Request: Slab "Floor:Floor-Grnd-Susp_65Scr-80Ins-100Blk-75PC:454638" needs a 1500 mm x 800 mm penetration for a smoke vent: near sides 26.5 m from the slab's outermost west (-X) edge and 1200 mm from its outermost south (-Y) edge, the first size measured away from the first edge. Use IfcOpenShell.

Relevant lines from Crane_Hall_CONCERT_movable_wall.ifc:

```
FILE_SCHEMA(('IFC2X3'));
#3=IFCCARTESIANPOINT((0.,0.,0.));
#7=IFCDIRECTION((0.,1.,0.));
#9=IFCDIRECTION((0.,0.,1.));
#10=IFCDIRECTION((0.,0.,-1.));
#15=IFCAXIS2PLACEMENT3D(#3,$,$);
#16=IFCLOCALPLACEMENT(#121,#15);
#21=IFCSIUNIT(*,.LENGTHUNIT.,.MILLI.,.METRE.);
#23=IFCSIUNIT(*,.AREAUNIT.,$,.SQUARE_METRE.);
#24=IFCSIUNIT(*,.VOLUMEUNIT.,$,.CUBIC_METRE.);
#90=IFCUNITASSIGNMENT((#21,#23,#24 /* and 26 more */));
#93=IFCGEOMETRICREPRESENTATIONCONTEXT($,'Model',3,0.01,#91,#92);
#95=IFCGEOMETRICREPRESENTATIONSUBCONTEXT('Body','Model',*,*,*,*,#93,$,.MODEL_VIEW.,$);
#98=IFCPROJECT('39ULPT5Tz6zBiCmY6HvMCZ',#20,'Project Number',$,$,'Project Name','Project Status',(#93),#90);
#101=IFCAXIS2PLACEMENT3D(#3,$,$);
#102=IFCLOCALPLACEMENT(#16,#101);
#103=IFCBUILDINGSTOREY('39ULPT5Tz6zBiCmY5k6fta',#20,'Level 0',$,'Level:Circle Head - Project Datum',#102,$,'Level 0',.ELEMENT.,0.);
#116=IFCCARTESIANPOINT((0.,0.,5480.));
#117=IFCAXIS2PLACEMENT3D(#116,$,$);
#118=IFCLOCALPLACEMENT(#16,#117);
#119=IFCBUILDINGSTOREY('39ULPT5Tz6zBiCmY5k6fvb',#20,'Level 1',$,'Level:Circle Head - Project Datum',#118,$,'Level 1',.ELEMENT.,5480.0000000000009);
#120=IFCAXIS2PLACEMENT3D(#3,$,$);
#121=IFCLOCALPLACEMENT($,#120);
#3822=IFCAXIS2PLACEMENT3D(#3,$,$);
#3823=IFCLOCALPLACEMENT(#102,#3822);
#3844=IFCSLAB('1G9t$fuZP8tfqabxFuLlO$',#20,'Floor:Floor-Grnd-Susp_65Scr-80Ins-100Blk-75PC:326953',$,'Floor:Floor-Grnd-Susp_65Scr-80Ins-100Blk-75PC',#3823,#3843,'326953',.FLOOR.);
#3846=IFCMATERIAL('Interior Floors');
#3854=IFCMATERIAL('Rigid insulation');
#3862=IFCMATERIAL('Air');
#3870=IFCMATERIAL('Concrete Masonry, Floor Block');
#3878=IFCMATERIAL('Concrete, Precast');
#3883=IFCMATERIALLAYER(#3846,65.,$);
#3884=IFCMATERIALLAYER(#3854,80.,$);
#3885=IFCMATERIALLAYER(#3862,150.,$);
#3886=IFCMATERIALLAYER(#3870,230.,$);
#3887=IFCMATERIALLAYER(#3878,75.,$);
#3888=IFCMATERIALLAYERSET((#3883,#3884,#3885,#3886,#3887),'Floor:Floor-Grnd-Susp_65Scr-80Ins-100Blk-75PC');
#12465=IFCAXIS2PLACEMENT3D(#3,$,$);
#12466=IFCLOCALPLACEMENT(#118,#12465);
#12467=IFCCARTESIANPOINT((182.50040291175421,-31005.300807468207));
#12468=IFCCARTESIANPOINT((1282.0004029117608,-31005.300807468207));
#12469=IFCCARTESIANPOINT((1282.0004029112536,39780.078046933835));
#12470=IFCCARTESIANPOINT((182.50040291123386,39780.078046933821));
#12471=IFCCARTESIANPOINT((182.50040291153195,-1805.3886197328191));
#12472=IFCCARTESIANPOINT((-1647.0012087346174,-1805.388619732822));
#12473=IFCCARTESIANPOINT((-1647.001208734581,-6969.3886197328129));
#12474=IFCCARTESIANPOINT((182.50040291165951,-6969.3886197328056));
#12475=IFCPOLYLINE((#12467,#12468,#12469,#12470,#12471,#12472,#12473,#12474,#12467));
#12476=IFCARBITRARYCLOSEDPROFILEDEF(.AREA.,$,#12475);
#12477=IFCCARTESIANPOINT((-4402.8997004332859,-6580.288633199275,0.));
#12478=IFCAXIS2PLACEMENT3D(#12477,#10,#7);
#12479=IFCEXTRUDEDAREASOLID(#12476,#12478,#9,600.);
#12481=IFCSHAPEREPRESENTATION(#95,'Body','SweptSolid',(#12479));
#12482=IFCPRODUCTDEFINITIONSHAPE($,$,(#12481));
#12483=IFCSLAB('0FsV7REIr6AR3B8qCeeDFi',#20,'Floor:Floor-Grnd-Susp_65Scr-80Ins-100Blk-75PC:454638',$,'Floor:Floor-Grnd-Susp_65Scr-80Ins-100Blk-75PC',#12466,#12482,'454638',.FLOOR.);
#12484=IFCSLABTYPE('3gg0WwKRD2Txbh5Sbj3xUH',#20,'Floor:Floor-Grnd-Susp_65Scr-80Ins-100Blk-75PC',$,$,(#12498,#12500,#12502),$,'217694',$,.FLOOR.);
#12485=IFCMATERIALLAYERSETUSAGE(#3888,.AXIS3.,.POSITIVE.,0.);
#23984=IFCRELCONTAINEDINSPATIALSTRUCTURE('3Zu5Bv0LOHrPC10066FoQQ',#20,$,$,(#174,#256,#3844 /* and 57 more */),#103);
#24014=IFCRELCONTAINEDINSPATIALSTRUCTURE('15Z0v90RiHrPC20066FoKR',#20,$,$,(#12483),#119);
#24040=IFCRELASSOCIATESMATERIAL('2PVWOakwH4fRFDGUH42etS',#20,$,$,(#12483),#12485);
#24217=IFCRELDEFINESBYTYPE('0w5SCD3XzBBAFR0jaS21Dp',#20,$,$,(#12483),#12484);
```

```python
import numpy as np
import ifcopenshell
import ifcopenshell.api.feature
import ifcopenshell.api.geometry
import ifcopenshell.api.root
import ifcopenshell.geom
import ifcopenshell.util.placement
import ifcopenshell.util.representation
import ifcopenshell.util.shape
import ifcopenshell.util.unit

model = ifcopenshell.open("Crane_Hall_CONCERT_movable_wall.ifc")
unit_scale = ifcopenshell.util.unit.calculate_unit_scale(model)
settings = ifcopenshell.geom.settings()


def volume(element):
    """Net volume in cubic metres, openings subtracted."""
    shape = ifcopenshell.geom.create_shape(settings, element)
    return ifcopenshell.util.shape.get_volume(shape.geometry)


slab = model.by_guid("0FsV7REIr6AR3B8qCeeDFi")
before = volume(slab)

# Extent in the slab's own axes, in metres. The edges named are its -X and -Y sides.
slab_shape = ifcopenshell.geom.create_shape(settings, slab)
vertices = ifcopenshell.util.shape.get_vertices(slab_shape.geometry)
x_min, y_min, bottom = vertices.min(axis=0)
top = vertices[:, 2].max()

opening = ifcopenshell.api.root.create_entity(model, ifc_class="IfcOpeningElement", name="Smoke vent opening")
context = ifcopenshell.util.representation.get_context(model, "Model", "Body", "MODEL_VIEW")
width, depth = 1.5, 0.8
outline = [(0.0, 0.0), (width, 0.0), (width, depth), (0.0, depth), (0.0, 0.0)]
# Overshoot both faces by 50 mm so the cut is clean.
shape = ifcopenshell.api.geometry.add_slab_representation(
    model, context=context, depth=top - bottom + 0.1, polyline=outline
)
ifcopenshell.api.geometry.assign_representation(model, product=opening, representation=shape)

matrix = ifcopenshell.util.placement.get_local_placement(slab.ObjectPlacement)
matrix[:, 3] = matrix @ np.append(np.array([x_min + 26.5, y_min + 1.2, bottom - 0.05]) / unit_scale, 1.0)
ifcopenshell.api.geometry.edit_object_placement(model, product=opening, matrix=matrix, is_si=False)
ifcopenshell.api.feature.add_feature(model, feature=opening, element=slab)

after = volume(slab)

print(f"slab volume {before:.3f} -> {after:.3f} m3")

model.write("Crane_Hall_CONCERT_movable_wall_v2.ifc")
```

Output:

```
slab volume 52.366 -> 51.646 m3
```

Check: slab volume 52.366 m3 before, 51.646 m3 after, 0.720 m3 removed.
